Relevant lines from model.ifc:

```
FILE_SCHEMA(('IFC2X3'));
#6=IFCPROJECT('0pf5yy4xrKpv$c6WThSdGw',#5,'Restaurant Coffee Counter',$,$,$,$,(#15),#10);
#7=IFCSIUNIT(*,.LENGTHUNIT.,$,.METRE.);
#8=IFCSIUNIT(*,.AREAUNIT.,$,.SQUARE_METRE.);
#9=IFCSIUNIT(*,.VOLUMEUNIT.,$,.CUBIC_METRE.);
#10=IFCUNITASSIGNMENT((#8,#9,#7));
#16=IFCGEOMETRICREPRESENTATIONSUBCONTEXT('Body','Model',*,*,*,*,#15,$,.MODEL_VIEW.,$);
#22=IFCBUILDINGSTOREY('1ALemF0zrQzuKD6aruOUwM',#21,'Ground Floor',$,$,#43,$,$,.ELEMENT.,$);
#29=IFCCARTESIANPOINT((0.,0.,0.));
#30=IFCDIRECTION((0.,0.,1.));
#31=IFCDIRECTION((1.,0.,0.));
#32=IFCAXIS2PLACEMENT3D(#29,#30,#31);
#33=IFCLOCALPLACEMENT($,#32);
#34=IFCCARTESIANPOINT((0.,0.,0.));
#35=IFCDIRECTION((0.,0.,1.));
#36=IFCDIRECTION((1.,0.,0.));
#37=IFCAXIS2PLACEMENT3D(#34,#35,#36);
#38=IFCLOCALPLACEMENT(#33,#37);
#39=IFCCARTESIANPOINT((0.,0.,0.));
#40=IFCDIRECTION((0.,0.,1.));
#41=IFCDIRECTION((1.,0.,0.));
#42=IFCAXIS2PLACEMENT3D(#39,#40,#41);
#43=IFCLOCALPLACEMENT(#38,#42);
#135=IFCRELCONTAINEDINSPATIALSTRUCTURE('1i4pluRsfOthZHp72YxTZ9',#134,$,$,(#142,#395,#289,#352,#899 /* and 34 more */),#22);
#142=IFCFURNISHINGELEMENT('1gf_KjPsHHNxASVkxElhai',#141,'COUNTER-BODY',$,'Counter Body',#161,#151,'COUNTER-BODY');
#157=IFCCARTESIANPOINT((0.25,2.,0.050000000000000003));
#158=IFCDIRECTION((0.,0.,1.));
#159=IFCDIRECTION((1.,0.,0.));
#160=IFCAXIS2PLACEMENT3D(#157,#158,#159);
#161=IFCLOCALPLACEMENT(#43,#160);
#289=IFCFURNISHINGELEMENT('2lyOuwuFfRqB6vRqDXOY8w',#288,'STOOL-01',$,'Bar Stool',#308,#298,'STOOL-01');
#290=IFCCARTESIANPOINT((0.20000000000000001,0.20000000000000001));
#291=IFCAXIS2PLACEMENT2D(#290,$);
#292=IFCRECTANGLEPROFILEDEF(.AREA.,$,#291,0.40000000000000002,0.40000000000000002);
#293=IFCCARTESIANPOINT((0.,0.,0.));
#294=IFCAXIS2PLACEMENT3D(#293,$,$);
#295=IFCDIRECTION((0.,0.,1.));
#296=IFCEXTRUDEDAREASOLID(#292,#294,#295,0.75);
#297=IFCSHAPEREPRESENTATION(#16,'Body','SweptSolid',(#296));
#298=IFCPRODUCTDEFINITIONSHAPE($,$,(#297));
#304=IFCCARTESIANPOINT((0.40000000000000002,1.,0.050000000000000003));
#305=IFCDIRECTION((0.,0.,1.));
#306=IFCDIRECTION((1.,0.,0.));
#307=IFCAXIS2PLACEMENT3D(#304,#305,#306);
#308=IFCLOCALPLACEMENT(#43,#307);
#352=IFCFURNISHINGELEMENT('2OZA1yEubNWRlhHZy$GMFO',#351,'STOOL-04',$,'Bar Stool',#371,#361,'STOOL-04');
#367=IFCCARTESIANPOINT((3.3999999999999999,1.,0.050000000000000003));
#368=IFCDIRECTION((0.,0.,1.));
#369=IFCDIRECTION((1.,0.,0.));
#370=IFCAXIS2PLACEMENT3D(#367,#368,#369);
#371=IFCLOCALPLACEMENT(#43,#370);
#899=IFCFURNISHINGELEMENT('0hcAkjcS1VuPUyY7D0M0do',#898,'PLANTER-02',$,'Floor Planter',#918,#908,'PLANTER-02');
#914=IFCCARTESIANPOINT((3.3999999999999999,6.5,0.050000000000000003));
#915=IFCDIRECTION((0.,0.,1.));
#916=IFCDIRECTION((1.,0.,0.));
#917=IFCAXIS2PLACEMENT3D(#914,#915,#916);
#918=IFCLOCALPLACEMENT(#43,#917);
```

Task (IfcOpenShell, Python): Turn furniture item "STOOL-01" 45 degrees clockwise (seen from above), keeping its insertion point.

```python
import ifcopenshell
import ifcopenshell.api.geometry
import ifcopenshell.util.placement

model = ifcopenshell.open("model.ifc")

item = model.by_id(289)
matrix = ifcopenshell.util.placement.get_local_placement(item.ObjectPlacement)
matrix = matrix @ ifcopenshell.util.placement.rotation(-45, "Z")
ifcopenshell.api.geometry.edit_object_placement(model, product=item, matrix=matrix, is_si=False)

print(ifcopenshell.util.placement.get_local_placement(item.ObjectPlacement).round(3) + 0.0)

model.write("model_v2.ifc")
```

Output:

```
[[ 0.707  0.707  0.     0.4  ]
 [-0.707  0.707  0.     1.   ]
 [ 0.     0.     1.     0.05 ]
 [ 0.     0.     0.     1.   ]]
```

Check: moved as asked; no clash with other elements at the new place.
